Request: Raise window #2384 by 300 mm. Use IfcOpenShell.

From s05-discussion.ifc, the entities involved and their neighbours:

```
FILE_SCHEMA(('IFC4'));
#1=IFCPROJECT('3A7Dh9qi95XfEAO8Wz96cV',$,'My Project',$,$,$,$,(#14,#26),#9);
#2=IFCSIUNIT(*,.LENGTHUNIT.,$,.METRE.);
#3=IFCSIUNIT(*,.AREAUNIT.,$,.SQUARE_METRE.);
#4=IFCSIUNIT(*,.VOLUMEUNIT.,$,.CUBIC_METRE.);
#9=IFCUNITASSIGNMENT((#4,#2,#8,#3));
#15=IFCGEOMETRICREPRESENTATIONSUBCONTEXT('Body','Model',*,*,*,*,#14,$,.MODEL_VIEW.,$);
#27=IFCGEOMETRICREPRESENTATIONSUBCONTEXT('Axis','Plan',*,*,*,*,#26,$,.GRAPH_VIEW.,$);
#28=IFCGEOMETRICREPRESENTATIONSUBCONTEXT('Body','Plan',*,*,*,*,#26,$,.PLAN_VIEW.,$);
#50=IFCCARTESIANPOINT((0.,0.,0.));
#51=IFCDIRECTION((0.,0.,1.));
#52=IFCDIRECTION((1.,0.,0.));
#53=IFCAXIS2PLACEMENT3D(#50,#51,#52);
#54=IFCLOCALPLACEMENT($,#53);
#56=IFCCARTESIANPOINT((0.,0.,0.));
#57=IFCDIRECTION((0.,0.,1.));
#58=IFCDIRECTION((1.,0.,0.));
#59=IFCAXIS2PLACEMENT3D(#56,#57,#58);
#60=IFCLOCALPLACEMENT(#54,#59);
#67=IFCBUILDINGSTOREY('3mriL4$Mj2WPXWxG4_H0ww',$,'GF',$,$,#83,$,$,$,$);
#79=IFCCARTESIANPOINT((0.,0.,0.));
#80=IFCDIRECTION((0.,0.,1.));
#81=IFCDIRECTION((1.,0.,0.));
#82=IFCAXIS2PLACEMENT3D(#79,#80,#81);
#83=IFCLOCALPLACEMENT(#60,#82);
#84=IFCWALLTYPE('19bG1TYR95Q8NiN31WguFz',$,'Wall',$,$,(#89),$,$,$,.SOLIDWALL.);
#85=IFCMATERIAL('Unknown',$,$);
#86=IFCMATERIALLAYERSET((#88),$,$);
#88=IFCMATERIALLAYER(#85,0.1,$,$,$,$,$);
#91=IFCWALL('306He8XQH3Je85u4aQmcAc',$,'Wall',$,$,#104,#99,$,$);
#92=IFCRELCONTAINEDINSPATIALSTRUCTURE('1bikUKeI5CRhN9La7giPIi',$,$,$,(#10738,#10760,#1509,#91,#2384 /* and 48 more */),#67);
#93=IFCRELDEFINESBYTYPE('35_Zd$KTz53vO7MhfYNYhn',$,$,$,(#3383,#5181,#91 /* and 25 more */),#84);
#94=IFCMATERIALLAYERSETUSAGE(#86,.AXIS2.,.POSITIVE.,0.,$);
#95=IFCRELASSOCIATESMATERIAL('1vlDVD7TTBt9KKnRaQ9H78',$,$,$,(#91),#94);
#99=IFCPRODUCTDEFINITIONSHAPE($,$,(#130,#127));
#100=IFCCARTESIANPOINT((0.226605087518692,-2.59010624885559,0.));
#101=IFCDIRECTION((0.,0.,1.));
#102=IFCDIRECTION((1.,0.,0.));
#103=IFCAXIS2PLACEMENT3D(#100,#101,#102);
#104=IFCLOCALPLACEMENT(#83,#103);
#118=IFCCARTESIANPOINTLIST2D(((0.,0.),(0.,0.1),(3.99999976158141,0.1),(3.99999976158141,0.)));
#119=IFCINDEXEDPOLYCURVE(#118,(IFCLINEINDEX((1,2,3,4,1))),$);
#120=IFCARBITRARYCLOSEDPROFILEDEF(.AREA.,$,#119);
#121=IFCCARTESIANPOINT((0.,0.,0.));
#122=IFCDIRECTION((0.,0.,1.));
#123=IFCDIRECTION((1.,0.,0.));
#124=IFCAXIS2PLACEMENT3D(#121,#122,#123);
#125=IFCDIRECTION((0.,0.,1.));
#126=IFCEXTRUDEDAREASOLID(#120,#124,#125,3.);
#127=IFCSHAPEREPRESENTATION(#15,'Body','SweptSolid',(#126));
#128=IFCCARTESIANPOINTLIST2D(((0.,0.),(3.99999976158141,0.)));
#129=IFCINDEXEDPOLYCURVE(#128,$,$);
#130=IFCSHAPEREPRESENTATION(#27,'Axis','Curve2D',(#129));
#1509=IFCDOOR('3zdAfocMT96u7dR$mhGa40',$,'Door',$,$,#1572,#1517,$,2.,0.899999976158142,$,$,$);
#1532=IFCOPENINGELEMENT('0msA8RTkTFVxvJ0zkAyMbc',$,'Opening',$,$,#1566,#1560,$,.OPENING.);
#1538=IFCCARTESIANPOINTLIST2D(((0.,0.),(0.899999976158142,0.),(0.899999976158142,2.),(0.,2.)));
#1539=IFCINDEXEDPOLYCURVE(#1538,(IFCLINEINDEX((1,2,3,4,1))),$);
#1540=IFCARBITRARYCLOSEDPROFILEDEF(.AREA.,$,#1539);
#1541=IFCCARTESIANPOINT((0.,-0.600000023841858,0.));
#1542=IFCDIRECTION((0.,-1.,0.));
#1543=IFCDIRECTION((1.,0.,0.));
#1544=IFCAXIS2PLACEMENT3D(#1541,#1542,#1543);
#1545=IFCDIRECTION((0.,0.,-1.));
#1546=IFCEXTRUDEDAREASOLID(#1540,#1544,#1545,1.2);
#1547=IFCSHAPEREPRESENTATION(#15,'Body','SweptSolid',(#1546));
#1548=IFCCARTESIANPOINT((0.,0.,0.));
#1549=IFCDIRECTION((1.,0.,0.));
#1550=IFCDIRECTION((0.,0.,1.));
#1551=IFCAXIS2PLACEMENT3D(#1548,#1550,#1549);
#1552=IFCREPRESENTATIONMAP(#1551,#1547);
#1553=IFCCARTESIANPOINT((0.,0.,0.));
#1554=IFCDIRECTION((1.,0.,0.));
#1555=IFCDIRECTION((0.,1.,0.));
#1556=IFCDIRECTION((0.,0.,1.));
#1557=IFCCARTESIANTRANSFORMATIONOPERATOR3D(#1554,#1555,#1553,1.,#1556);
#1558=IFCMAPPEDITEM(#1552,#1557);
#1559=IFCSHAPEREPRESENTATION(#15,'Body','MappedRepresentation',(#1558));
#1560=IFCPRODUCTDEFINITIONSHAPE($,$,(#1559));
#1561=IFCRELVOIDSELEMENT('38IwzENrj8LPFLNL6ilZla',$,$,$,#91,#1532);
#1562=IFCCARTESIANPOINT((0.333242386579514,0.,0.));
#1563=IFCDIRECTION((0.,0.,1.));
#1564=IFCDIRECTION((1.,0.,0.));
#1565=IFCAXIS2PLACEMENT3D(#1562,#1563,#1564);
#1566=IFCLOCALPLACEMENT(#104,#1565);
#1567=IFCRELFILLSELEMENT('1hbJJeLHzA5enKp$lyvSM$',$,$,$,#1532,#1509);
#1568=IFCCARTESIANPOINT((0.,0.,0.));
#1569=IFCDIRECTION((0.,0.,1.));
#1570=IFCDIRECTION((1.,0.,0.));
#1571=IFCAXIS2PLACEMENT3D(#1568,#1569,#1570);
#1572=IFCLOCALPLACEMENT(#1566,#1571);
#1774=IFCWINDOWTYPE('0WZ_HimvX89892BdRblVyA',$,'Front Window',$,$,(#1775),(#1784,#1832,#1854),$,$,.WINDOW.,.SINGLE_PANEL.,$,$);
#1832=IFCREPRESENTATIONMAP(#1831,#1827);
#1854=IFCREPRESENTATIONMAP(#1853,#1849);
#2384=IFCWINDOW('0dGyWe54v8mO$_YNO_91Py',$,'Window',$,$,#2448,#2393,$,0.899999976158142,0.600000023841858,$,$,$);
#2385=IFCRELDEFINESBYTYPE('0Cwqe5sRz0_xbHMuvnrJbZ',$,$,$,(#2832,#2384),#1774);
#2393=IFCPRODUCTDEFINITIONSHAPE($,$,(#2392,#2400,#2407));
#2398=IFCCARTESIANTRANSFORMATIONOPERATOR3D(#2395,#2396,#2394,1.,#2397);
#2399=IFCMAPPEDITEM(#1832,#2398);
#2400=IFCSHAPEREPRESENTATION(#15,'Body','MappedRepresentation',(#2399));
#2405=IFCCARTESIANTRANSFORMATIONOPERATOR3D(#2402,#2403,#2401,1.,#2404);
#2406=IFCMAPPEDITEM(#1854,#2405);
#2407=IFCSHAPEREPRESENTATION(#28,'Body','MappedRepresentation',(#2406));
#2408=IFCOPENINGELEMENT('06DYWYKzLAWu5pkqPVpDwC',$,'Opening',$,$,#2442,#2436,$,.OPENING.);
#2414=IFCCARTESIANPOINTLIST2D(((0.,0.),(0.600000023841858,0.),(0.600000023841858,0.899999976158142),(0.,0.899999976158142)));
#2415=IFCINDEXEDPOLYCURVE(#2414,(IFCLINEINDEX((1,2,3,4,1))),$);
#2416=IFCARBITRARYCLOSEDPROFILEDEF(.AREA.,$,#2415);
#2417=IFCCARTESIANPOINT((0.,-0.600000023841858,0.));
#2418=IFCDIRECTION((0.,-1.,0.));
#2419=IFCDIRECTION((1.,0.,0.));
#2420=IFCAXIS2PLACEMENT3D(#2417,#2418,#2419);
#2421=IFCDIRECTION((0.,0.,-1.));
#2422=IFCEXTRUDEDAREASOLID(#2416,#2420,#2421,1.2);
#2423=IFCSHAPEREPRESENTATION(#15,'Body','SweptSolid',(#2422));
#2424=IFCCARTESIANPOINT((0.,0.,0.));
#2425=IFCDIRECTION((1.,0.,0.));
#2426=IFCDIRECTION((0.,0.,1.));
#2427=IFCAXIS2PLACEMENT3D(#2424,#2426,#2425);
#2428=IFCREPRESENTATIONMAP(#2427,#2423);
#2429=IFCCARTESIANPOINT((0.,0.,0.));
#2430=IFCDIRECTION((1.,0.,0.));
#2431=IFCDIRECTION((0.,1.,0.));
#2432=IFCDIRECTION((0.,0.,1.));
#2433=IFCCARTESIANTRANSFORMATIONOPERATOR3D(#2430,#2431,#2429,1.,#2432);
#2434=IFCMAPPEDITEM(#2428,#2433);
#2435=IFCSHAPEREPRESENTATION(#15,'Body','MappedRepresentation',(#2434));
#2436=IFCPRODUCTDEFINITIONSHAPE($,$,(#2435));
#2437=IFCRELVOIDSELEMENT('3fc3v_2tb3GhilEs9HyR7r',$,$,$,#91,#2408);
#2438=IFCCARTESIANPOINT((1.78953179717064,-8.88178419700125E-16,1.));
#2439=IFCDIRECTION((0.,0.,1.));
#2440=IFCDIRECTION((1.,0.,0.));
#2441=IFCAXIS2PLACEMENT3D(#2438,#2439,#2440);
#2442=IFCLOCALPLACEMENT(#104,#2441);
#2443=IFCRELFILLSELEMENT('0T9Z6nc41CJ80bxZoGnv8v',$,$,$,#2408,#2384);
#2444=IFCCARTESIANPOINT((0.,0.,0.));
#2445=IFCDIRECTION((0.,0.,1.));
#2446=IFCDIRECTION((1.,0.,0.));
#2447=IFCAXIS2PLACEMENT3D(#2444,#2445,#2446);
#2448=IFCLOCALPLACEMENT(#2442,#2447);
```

```python
import numpy as np
import ifcopenshell
import ifcopenshell.api.geometry
import ifcopenshell.util.placement
import ifcopenshell.util.unit

model = ifcopenshell.open("s05-discussion.ifc")
unit_scale = ifcopenshell.util.unit.calculate_unit_scale(model)

window = model.by_id(2384)
opening = window.FillsVoids[0].RelatingOpeningElement
dz = 0.3 / unit_scale

shift = np.array([0.0, 0.0, dz])
# The window is placed relative to its opening, so it follows when the opening moves.
matrix = ifcopenshell.util.placement.get_local_placement(opening.ObjectPlacement)
matrix[:3, 3] += shift
ifcopenshell.api.geometry.edit_object_placement(
    model, product=opening, matrix=matrix, is_si=False, should_transform_children=True
)

print(f"moved by {dz * unit_scale:+.3f} m")

model.write("s05-discussion_edited.ifc")
```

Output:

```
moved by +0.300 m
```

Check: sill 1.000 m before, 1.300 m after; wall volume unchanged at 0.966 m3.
